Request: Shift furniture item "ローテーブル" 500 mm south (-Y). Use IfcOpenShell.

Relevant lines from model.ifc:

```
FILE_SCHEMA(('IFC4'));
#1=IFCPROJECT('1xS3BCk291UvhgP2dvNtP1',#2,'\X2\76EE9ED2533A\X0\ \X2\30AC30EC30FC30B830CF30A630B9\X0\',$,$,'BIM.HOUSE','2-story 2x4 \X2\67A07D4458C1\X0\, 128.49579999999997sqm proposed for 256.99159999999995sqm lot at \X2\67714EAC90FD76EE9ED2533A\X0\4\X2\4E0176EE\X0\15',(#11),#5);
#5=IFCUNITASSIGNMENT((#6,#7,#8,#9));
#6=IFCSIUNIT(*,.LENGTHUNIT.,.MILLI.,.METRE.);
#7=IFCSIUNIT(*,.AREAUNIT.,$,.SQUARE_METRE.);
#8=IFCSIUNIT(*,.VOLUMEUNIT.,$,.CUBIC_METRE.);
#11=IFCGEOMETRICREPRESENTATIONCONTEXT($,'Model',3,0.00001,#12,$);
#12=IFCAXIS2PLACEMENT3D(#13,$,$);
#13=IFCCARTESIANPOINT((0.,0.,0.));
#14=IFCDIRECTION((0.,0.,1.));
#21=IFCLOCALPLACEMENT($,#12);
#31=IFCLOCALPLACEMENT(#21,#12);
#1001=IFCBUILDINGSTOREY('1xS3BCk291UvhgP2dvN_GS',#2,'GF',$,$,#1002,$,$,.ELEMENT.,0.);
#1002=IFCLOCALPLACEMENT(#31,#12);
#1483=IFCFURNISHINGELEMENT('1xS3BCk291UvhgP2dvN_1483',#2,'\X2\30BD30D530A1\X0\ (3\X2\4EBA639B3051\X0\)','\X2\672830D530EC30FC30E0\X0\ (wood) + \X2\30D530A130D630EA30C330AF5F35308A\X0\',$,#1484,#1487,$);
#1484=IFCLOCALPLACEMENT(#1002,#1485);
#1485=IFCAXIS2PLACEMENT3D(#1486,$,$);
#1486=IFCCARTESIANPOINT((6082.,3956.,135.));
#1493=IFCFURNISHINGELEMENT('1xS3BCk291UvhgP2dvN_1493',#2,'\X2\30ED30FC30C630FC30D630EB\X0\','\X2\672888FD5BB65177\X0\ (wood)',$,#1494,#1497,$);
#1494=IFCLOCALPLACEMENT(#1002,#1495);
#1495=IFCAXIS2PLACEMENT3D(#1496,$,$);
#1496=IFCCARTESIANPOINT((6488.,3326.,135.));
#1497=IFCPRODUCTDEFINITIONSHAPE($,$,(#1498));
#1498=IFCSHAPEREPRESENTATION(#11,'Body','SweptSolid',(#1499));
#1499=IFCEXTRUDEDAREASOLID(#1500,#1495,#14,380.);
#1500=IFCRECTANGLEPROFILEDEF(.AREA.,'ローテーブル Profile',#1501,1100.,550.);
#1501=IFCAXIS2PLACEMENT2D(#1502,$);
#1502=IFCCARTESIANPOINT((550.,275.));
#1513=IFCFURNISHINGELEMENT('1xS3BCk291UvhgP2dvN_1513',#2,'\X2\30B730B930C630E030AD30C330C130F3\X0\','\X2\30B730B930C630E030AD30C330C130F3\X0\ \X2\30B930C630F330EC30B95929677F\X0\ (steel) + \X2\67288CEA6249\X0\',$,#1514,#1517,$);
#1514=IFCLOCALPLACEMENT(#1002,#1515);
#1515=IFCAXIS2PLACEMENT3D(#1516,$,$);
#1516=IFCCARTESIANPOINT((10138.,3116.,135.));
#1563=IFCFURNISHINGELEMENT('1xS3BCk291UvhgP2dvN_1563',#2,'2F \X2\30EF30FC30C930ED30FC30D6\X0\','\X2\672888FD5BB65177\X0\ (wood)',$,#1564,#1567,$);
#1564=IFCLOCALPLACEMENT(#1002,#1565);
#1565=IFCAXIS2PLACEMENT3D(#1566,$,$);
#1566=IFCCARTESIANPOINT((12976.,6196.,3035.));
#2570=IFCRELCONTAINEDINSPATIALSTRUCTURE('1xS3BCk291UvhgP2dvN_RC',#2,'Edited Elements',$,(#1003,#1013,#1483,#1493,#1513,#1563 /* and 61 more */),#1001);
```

```python
import ifcopenshell
import ifcopenshell.api.geometry
import ifcopenshell.util.placement
import ifcopenshell.util.unit

model = ifcopenshell.open("model.ifc")
unit_scale = ifcopenshell.util.unit.calculate_unit_scale(model)

item = model.by_guid("1xS3BCk291UvhgP2dvN_1493")
matrix = ifcopenshell.util.placement.get_local_placement(item.ObjectPlacement)
matrix[1, 3] -= 0.5 / unit_scale
ifcopenshell.api.geometry.edit_object_placement(model, product=item, matrix=matrix, is_si=False)

print(ifcopenshell.util.placement.get_local_placement(item.ObjectPlacement).round(3) + 0.0)

model.write("model_v2.ifc")
```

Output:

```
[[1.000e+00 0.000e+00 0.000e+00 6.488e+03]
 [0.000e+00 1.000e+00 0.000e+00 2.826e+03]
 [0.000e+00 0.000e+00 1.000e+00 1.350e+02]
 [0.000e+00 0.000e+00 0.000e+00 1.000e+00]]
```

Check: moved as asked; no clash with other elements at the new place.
